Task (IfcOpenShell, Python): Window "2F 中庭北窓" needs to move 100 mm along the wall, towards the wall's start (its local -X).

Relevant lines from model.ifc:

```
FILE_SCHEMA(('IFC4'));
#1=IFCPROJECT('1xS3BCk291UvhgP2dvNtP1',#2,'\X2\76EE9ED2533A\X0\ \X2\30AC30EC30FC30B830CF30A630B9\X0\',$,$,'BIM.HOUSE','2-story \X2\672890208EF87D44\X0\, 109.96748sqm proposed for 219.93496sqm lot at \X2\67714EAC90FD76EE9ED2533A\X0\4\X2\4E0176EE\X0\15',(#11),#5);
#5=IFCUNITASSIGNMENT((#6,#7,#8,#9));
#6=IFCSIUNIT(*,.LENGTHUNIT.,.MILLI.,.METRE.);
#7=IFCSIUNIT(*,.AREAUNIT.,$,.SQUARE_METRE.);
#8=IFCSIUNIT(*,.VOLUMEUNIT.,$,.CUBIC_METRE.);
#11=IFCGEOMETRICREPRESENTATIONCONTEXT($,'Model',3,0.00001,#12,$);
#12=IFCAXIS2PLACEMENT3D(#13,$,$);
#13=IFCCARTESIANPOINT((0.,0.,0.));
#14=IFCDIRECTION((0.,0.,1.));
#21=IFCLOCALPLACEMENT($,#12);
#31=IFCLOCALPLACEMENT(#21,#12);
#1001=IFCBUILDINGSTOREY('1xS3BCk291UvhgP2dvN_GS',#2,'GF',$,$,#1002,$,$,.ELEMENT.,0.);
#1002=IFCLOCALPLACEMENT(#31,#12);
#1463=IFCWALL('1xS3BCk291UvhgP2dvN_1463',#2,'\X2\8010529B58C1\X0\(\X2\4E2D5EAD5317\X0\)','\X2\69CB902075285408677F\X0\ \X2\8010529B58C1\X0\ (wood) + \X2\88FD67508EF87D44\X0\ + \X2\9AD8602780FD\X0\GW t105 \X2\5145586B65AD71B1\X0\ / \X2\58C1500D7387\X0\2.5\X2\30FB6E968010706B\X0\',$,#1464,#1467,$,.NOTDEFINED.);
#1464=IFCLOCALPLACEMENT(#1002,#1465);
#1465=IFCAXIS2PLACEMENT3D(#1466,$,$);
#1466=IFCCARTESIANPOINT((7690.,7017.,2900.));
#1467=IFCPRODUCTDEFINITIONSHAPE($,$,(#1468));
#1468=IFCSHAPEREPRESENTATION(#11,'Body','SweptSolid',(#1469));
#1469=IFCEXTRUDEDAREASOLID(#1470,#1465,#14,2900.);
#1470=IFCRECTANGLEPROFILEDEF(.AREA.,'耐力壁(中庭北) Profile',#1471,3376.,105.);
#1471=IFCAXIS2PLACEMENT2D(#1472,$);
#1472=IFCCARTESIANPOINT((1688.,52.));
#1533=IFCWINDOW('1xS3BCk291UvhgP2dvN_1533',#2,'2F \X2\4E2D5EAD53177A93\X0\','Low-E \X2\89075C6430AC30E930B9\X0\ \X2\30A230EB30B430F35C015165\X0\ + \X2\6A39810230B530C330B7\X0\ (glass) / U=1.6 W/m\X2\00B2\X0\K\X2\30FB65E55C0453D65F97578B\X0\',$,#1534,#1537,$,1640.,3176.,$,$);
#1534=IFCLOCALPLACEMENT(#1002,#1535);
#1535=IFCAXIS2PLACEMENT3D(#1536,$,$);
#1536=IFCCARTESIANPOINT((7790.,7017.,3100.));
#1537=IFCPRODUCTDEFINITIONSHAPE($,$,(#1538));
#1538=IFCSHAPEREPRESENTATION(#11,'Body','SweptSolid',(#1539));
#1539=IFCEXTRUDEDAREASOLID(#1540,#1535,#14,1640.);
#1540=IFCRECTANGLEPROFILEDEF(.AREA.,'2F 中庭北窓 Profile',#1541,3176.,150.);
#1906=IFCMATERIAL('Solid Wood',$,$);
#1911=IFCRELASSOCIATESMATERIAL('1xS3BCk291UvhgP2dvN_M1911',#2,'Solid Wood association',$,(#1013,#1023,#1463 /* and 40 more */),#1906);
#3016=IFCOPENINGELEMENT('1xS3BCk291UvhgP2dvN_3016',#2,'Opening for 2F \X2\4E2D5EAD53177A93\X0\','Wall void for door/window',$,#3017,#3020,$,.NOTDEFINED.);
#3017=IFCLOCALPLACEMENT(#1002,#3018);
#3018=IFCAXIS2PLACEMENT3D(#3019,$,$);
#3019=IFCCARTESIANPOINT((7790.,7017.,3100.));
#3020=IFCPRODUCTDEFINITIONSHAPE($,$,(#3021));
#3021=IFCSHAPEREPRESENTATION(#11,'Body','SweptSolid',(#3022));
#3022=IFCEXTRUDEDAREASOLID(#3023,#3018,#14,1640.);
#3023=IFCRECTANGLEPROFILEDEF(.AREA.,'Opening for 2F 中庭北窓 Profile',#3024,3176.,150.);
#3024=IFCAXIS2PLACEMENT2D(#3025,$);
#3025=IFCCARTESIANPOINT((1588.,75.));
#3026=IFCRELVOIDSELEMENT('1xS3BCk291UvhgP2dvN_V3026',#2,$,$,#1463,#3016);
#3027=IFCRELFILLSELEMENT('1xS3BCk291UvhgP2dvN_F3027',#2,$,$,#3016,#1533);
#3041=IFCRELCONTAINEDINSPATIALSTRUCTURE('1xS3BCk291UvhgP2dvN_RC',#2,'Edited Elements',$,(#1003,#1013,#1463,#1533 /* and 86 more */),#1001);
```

```python
import ifcopenshell
import ifcopenshell.api.geometry
import ifcopenshell.util.placement
import ifcopenshell.util.unit

model = ifcopenshell.open("model.ifc")
unit_scale = ifcopenshell.util.unit.calculate_unit_scale(model)

window = model.by_guid("1xS3BCk291UvhgP2dvN_1533")
opening = window.FillsVoids[0].RelatingOpeningElement
wall = opening.VoidsElements[0].RelatingBuildingElement

wall_matrix = ifcopenshell.util.placement.get_local_placement(wall.ObjectPlacement)
shift = wall_matrix[:3, 0] * -0.1 / unit_scale
before = ifcopenshell.util.placement.get_local_placement(window.ObjectPlacement)[:3, 3].copy()

# The window is not placed relative to its opening, so move both.
for product in (opening, window):
    matrix = ifcopenshell.util.placement.get_local_placement(product.ObjectPlacement)
    matrix[:3, 3] += shift
    ifcopenshell.api.geometry.edit_object_placement(model, product=product, matrix=matrix, is_si=False)

after = ifcopenshell.util.placement.get_local_placement(window.ObjectPlacement)[:3, 3]
print("window moved by", (after - before).round(3) + 0.0)

model.write("model_edited.ifc")
```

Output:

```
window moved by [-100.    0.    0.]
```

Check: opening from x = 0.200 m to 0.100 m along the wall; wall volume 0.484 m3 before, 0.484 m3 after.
